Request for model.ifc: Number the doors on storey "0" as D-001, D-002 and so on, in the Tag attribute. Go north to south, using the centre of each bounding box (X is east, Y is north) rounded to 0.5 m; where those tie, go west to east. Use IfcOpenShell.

First a look at what the model holds.

```python
import ifcopenshell
import ifcopenshell.util.element
import ifcopenshell.util.placement

model = ifcopenshell.open("model.ifc")
print(model.schema)
storey = next(s for s in model.by_type("IfcBuildingStorey") if s.Name == "0")
doors = [e for e in ifcopenshell.util.element.get_decomposition(storey) if e.is_a("IfcDoor")]
for e in sorted(doors, key=lambda e: e.id()):
    origin = ifcopenshell.util.placement.get_local_placement(e.ObjectPlacement)[:3, 3]
    print(e.id(), e.Tag, e.Name, origin.round(2) + 0.0, sep=" | ")
```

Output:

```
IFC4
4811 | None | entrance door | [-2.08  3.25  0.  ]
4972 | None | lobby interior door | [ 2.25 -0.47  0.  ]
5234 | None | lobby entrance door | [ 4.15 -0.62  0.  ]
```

```python
import ifcopenshell
import ifcopenshell.geom
import ifcopenshell.util.element
import ifcopenshell.util.shape

model = ifcopenshell.open("model.ifc")
settings = ifcopenshell.geom.settings()
settings.set("use-world-coords", True)


def centre(element):
    shape = ifcopenshell.geom.create_shape(settings, element)
    return ifcopenshell.util.shape.get_bbox_centroid(shape.geometry)


storey = next(s for s in model.by_type("IfcBuildingStorey") if s.Name == "0")
doors = [e for e in ifcopenshell.util.element.get_decomposition(storey) if e.is_a("IfcDoor")]

# Insertion points can sit at a corner or the storey origin, so sort by the geometry (in metres).
centres = {e: centre(e) for e in doors}
doors.sort(key=lambda e: (-round(centres[e][1] / 0.5), centres[e][0]))

for i, e in enumerate(doors, start=1):
    number = f"D-0{i:02d}"
    e.Tag = number
    print(e.id(), number)

model.write("model_updated.ifc")
```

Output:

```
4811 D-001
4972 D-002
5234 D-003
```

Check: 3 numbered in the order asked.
